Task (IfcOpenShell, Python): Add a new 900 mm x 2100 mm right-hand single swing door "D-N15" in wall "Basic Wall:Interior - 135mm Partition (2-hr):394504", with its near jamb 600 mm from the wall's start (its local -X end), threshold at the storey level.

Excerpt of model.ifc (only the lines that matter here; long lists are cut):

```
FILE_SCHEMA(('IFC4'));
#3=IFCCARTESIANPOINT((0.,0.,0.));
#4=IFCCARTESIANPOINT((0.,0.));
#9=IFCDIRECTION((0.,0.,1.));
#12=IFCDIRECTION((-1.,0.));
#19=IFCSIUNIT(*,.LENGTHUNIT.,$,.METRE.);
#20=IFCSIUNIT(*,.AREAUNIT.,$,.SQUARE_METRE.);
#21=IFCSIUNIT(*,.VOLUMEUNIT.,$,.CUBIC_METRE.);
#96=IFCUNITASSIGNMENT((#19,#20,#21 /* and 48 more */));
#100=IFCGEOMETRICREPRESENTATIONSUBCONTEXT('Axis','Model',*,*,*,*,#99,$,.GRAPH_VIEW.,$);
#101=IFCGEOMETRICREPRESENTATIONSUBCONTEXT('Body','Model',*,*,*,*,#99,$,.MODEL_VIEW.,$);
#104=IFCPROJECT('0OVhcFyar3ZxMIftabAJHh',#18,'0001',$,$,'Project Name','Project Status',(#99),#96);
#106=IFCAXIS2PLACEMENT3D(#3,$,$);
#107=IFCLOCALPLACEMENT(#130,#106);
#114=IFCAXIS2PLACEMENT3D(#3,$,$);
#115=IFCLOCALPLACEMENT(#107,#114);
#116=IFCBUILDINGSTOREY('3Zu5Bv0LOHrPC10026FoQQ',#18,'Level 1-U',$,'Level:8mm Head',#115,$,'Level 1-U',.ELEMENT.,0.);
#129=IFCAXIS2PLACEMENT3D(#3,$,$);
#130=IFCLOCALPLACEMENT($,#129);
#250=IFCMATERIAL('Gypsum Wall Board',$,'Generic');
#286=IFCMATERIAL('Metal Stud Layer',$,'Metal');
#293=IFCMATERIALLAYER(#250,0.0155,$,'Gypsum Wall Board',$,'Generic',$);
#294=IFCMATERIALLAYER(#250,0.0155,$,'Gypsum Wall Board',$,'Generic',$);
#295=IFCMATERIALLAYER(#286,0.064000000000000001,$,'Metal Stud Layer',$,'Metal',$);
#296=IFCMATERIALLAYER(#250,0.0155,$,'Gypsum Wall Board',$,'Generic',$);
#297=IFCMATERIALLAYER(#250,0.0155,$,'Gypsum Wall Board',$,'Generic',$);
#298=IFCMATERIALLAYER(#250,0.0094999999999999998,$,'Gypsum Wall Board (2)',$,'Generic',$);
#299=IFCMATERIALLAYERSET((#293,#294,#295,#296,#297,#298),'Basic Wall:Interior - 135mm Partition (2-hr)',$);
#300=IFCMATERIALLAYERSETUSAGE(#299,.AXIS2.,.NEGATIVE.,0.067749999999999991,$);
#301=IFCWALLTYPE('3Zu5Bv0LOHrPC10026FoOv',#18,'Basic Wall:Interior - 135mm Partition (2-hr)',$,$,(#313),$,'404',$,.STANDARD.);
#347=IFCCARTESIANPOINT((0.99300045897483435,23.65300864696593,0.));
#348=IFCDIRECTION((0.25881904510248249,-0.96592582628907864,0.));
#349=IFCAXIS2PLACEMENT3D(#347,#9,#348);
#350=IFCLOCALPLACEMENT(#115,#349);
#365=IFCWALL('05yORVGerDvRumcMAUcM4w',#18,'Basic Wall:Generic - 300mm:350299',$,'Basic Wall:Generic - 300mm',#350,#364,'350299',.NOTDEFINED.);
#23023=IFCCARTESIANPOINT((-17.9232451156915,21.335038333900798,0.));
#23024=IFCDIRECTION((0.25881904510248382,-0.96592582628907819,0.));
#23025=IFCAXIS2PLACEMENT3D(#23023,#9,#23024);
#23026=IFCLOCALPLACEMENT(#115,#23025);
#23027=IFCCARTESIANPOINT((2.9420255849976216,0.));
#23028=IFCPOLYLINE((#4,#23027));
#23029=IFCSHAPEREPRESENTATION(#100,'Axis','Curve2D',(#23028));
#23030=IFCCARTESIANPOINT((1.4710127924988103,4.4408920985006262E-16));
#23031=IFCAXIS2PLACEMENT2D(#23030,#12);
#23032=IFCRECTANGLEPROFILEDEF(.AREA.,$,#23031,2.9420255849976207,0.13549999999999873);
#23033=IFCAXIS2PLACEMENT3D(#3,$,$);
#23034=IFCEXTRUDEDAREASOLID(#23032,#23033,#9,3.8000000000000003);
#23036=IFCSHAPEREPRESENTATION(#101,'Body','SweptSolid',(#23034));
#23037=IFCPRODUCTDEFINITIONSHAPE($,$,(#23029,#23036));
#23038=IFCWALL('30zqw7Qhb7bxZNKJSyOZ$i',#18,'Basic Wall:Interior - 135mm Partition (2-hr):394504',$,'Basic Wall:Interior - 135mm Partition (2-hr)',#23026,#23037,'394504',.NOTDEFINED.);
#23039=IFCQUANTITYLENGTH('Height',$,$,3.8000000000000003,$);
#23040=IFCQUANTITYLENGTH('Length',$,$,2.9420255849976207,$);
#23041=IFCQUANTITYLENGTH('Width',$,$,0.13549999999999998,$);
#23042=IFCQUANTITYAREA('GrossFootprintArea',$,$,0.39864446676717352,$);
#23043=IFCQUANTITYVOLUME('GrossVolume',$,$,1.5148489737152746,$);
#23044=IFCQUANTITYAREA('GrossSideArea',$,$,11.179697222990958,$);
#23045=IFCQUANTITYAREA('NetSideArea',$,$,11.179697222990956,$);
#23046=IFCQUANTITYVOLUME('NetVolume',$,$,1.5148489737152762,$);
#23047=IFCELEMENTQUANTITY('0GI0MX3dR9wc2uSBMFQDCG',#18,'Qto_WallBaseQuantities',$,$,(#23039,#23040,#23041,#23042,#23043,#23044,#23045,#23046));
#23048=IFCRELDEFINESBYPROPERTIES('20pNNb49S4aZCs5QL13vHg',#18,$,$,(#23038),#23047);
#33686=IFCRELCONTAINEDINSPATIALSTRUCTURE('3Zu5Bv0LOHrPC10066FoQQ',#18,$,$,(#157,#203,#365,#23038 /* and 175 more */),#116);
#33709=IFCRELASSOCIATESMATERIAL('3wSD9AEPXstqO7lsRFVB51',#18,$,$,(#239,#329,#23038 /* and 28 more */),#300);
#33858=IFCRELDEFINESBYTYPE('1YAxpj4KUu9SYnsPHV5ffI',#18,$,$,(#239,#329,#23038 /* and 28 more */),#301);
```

```python
import numpy as np
import ifcopenshell
import ifcopenshell.api.feature
import ifcopenshell.api.geometry
import ifcopenshell.api.pset
import ifcopenshell.api.root
import ifcopenshell.api.spatial
import ifcopenshell.geom
import ifcopenshell.util.element
import ifcopenshell.util.placement
import ifcopenshell.util.representation
import ifcopenshell.util.shape
import ifcopenshell.util.unit

model = ifcopenshell.open("model.ifc")
unit_scale = ifcopenshell.util.unit.calculate_unit_scale(model)
area_scale = ifcopenshell.util.unit.calculate_unit_scale(model, "AREAUNIT")
volume_scale = ifcopenshell.util.unit.calculate_unit_scale(model, "VOLUMEUNIT")
settings = ifcopenshell.geom.settings()


def volume(element):
    """Net volume in cubic metres, openings subtracted."""
    shape = ifcopenshell.geom.create_shape(settings, element)
    return ifcopenshell.util.shape.get_volume(shape.geometry)


wall = model.by_guid("30zqw7Qhb7bxZNKJSyOZ$i")
storey = ifcopenshell.util.element.get_container(wall, ifc_class="IfcBuildingStorey")
context = ifcopenshell.util.representation.get_context(model, "Model", "Body", "MODEL_VIEW")
before = volume(wall)

width, height, from_end, sill = 0.9, 2.1, 0.6, 0.0  # metres

# The wall runs along its own X axis, and the end named is its -X end.
wall_shape = ifcopenshell.geom.create_shape(settings, wall)
x, y, z = ifcopenshell.util.shape.get_vertices(wall_shape.geometry).T
start = x.min() + from_end
face, thickness = float(y.min()), float(y.max() - y.min())
wall_matrix = ifcopenshell.util.placement.get_local_placement(wall.ObjectPlacement)
level = ifcopenshell.util.placement.get_local_placement(storey.ObjectPlacement)[2, 3]


def in_wall(x, y):
    """Placement at x, y metres in the wall's axes, at sill height."""
    matrix = wall_matrix.copy()
    matrix[:, 3] = wall_matrix @ np.array([x / unit_scale, y / unit_scale, 0.0, 1.0])
    matrix[2, 3] = level + sill / unit_scale
    return matrix


# Opening: a box that overshoots both wall faces by 50 mm.
opening = ifcopenshell.api.root.create_entity(model, ifc_class="IfcOpeningElement", predefined_type="OPENING")
box = ifcopenshell.api.geometry.add_wall_representation(
    model, context=context, length=width, height=height, thickness=thickness + 0.1
)
ifcopenshell.api.geometry.assign_representation(model, product=opening, representation=box)
ifcopenshell.api.geometry.edit_object_placement(model, product=opening, matrix=in_wall(start, face - 0.05), is_si=False)
ifcopenshell.api.feature.add_feature(model, feature=opening, element=wall)

door = ifcopenshell.api.root.create_entity(model, ifc_class="IfcDoor", name="D-N15", predefined_type="DOOR")
door.OverallWidth, door.OverallHeight = width / unit_scale, height / unit_scale
door.OperationType = "SINGLE_SWING_RIGHT"
body = ifcopenshell.api.geometry.add_door_representation(
    model,
    context=context,
    overall_width=door.OverallWidth,
    overall_height=door.OverallHeight,
    operation_type="SINGLE_SWING_RIGHT",
    lining_properties={"LiningDepth": thickness / unit_scale, "ThresholdDepth": thickness / unit_scale},
)
ifcopenshell.api.geometry.assign_representation(model, product=door, representation=body)
ifcopenshell.api.spatial.assign_container(model, products=[door], relating_structure=storey)
ifcopenshell.api.feature.add_filling(model, opening=opening, element=door)

# The lining spans the wall, so the door starts at the wall face.
ifcopenshell.api.geometry.edit_object_placement(model, product=door, matrix=in_wall(start, face), is_si=False)

after = volume(wall)

# Update the wall's stored quantities.
qto = model.by_id(ifcopenshell.util.element.get_pset(wall, "Qto_WallBaseQuantities", should_inherit=False)["id"])
ifcopenshell.api.pset.edit_qto(model, qto=qto, properties={
    "NetSideArea": after / thickness / area_scale,
    "NetVolume": after / volume_scale,
})

print(f"wall volume {before:.3f} -> {after:.3f} m3")

model.write("model_v2.ifc")
```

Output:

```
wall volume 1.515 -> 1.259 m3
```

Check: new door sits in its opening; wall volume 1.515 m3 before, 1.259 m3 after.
